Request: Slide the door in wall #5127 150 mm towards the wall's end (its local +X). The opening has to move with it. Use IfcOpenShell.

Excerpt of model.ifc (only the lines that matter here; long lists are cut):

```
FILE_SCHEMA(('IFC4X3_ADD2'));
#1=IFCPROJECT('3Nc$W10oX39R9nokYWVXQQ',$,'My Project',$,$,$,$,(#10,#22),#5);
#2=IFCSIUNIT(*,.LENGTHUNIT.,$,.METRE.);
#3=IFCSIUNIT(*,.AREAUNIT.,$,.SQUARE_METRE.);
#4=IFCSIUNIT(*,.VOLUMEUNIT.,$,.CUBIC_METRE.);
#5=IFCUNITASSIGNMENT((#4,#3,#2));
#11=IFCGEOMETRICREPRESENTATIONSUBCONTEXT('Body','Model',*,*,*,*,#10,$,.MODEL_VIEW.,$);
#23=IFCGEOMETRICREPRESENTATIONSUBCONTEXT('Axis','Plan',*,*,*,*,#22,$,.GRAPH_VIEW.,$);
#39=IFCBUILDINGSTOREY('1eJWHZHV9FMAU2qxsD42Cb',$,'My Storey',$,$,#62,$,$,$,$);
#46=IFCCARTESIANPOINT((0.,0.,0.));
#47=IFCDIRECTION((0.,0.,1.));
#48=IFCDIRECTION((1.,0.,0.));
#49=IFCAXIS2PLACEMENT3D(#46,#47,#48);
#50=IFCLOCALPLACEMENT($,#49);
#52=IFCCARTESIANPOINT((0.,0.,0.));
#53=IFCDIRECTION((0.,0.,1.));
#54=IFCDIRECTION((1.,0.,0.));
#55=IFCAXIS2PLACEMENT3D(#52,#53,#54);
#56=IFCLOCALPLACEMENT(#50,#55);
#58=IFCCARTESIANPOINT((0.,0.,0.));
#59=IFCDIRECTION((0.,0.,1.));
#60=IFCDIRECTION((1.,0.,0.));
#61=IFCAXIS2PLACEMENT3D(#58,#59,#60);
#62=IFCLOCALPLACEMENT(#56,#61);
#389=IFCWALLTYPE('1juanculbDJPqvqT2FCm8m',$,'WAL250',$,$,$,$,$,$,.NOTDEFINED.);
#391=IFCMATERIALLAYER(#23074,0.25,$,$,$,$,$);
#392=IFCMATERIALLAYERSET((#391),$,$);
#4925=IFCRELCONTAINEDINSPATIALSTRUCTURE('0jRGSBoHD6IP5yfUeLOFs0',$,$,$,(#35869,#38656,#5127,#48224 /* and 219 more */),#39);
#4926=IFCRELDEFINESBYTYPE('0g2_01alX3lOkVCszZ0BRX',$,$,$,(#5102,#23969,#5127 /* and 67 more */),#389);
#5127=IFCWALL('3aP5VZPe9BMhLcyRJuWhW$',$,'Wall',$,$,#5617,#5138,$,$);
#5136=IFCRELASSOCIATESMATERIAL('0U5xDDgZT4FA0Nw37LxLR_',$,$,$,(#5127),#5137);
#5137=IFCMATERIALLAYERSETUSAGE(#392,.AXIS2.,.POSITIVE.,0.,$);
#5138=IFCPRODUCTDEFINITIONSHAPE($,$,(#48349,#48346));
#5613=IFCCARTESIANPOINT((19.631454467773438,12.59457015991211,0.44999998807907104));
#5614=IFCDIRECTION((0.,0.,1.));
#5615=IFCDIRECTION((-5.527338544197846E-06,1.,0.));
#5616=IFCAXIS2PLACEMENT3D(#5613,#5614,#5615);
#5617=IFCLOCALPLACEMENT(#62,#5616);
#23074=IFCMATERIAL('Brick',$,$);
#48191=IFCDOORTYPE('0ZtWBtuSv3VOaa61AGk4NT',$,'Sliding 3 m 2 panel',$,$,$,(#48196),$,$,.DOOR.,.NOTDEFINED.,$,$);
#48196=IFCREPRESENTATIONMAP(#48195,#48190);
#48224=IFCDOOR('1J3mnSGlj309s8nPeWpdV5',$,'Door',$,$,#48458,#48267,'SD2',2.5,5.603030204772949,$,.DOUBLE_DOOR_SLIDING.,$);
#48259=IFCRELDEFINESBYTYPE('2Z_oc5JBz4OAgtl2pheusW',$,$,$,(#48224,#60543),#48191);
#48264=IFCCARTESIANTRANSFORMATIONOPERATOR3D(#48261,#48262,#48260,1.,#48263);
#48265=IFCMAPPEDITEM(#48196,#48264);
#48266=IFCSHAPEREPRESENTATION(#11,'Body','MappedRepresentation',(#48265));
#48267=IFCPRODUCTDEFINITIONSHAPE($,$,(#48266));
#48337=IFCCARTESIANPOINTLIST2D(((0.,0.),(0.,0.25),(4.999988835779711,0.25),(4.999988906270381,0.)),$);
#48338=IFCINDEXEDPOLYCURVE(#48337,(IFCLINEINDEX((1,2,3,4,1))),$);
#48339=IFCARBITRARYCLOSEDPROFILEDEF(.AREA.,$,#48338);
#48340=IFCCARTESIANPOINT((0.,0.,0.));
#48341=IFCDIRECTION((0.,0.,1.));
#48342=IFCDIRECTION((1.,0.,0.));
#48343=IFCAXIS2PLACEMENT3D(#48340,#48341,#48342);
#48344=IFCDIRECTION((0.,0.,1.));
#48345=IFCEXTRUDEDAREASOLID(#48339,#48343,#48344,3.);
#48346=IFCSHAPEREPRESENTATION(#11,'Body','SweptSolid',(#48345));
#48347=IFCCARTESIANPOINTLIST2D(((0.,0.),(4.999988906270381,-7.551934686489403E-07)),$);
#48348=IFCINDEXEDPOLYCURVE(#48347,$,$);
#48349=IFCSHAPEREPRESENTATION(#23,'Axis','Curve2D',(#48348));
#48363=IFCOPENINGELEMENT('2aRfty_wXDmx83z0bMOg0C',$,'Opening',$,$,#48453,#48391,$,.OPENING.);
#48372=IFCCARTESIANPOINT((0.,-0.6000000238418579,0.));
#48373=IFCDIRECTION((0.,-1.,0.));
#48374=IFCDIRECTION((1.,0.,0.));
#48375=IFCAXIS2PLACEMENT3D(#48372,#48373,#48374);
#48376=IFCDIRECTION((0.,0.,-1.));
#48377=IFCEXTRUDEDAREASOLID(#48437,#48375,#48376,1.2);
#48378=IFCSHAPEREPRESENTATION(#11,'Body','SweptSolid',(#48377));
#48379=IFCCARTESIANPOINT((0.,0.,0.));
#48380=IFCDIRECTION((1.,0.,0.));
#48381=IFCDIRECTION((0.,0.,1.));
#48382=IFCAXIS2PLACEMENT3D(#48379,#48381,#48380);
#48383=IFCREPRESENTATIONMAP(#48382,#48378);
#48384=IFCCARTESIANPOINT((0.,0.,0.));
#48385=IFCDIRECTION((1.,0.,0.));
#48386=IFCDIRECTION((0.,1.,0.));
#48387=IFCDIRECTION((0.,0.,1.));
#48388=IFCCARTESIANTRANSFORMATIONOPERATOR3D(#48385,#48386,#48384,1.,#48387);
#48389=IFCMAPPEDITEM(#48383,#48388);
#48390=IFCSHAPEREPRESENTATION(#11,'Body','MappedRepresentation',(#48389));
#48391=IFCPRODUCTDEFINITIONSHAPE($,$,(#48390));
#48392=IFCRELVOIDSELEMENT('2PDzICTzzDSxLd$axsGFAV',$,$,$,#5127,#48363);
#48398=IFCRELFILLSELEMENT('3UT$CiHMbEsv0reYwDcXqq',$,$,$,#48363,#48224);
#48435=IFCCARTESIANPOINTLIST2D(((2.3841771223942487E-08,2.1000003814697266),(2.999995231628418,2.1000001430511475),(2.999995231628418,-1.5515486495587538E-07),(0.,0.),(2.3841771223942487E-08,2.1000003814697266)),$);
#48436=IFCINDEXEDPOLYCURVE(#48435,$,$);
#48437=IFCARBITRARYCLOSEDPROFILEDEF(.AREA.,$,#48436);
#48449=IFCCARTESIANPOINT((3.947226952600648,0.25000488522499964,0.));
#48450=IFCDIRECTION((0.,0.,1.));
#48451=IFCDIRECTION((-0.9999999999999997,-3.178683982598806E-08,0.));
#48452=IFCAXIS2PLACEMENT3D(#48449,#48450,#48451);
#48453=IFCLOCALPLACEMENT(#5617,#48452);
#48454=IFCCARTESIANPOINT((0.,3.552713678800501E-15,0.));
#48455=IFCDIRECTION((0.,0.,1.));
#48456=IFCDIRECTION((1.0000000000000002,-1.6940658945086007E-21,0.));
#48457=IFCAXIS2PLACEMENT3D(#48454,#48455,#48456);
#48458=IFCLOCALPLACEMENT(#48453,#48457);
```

```python
import ifcopenshell
import ifcopenshell.api.geometry
import ifcopenshell.util.placement
import ifcopenshell.util.unit

model = ifcopenshell.open("model.ifc")
unit_scale = ifcopenshell.util.unit.calculate_unit_scale(model)

door = model.by_guid("1J3mnSGlj309s8nPeWpdV5")
opening = door.FillsVoids[0].RelatingOpeningElement
wall = opening.VoidsElements[0].RelatingBuildingElement

wall_matrix = ifcopenshell.util.placement.get_local_placement(wall.ObjectPlacement)
shift = wall_matrix[:3, 0] * 0.15 / unit_scale
before = ifcopenshell.util.placement.get_local_placement(door.ObjectPlacement)[:3, 3].copy()

# The door is placed relative to its opening, so it follows when the opening moves.
matrix = ifcopenshell.util.placement.get_local_placement(opening.ObjectPlacement)
matrix[:3, 3] += shift
ifcopenshell.api.geometry.edit_object_placement(
    model, product=opening, matrix=matrix, is_si=False, should_transform_children=True
)

after = ifcopenshell.util.placement.get_local_placement(door.ObjectPlacement)[:3, 3]
print("door moved by", (after - before).round(3) + 0.0)

model.write("model_v2.ifc")
```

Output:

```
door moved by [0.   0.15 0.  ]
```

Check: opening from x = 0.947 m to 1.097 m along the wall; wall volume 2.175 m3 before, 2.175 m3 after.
